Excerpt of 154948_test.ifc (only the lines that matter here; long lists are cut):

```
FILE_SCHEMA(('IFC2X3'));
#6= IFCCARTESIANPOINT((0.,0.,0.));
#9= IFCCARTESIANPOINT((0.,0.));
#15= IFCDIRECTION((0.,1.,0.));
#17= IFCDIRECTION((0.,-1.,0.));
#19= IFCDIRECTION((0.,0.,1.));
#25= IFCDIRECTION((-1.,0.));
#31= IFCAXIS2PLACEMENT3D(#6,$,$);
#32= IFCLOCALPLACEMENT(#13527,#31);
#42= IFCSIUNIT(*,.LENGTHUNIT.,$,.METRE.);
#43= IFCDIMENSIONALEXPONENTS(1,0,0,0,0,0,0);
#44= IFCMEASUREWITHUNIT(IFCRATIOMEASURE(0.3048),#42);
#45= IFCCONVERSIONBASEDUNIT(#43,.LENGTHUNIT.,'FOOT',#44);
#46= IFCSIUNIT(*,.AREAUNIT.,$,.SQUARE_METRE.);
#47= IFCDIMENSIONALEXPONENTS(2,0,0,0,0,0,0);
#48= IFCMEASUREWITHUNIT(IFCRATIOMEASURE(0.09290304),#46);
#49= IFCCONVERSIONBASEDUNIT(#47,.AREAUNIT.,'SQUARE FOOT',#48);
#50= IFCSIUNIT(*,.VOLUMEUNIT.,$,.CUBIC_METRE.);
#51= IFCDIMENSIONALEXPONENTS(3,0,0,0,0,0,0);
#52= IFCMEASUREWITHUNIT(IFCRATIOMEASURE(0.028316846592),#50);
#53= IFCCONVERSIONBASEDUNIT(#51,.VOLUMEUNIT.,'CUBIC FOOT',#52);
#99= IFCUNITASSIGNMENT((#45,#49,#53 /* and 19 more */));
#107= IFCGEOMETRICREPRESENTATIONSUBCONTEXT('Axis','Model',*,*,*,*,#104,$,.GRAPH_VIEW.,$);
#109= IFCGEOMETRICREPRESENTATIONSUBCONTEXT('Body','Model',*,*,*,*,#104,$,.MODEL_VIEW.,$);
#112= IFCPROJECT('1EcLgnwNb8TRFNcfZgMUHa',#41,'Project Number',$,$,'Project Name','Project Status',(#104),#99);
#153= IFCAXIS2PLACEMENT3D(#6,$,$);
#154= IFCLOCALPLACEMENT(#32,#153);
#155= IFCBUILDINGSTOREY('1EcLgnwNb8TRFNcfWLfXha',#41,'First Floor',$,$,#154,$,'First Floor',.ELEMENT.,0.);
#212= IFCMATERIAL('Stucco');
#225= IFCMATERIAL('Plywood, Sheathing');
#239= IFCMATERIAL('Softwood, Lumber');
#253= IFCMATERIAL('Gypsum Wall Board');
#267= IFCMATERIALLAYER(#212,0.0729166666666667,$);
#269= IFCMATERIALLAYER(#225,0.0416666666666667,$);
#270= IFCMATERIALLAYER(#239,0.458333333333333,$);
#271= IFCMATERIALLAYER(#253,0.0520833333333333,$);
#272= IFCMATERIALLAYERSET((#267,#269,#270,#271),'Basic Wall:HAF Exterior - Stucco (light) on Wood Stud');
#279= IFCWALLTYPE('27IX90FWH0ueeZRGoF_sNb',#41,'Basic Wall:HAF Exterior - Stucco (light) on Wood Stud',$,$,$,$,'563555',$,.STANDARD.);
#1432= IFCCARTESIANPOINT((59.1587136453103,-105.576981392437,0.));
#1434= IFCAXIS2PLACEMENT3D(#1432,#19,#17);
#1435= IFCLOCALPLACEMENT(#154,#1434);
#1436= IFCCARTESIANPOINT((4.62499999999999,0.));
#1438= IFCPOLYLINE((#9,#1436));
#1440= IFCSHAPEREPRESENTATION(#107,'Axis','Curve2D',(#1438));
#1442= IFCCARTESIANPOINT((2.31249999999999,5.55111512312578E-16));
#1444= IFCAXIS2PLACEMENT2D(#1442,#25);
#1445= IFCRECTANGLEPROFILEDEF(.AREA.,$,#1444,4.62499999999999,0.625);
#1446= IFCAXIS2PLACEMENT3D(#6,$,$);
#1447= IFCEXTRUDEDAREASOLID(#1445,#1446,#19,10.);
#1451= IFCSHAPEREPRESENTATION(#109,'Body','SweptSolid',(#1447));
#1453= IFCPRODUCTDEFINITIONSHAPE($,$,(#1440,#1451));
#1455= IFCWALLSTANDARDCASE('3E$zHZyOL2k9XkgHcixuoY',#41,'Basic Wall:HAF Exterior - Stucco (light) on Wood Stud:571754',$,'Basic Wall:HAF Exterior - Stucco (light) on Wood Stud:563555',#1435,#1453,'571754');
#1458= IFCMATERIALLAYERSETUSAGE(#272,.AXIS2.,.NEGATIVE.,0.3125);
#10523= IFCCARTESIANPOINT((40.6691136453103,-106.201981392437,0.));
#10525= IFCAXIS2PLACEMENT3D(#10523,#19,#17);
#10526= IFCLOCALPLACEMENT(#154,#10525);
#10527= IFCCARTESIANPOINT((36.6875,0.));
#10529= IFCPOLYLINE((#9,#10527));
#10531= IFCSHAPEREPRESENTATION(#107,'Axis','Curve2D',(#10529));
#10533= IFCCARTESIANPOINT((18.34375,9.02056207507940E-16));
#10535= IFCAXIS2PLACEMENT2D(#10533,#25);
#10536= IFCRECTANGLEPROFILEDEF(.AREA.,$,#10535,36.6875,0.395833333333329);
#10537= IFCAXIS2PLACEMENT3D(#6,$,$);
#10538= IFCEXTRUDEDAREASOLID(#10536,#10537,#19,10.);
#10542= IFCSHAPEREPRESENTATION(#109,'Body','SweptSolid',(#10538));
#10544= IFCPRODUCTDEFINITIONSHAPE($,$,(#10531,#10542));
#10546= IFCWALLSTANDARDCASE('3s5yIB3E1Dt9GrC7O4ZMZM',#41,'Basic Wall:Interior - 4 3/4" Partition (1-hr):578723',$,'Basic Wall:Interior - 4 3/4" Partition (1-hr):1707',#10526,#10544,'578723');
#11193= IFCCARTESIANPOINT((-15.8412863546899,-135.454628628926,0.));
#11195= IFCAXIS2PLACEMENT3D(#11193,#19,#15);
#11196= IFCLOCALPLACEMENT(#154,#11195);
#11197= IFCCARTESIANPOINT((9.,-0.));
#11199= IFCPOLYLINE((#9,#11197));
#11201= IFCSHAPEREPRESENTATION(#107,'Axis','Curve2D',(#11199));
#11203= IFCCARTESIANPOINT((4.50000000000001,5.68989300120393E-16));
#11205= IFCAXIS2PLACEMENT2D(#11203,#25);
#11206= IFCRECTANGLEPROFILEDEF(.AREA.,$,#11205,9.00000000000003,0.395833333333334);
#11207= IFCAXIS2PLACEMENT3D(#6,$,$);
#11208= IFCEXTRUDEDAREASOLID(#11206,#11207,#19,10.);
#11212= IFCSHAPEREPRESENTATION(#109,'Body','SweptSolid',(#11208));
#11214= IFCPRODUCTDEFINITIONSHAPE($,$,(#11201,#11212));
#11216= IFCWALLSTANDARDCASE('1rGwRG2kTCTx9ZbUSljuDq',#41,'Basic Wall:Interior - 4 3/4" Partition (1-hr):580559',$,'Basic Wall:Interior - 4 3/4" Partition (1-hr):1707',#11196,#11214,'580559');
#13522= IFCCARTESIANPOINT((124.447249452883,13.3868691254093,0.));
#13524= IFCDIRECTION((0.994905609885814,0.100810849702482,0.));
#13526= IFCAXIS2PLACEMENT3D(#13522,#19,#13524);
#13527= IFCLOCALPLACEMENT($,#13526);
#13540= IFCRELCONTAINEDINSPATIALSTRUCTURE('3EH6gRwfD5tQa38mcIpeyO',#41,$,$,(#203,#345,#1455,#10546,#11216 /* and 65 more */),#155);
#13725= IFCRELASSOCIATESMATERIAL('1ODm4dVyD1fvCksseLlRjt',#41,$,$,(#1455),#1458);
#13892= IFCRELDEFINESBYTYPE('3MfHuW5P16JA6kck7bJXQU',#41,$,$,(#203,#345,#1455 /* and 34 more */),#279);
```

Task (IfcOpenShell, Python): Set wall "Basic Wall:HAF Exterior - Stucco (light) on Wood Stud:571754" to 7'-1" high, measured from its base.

```python
import ifcopenshell
import ifcopenshell.geom
import ifcopenshell.util.representation
import ifcopenshell.util.shape
import ifcopenshell.util.unit

model = ifcopenshell.open("154948_test.ifc")
unit_scale = ifcopenshell.util.unit.calculate_unit_scale(model)
settings = ifcopenshell.geom.settings()


def volume(element):
    """Net volume in cubic metres, openings subtracted."""
    shape = ifcopenshell.geom.create_shape(settings, element)
    return ifcopenshell.util.shape.get_volume(shape.geometry)


wall = model.by_guid("3E$zHZyOL2k9XkgHcixuoY")
before = volume(wall)

body = ifcopenshell.util.representation.get_representation(wall, "Model", "Body")
solid = body.Items[0]
old_height = solid.Depth
solid.Depth = 85 * 0.0254 / unit_scale
after = volume(wall)

print(f"height {old_height:g} -> {solid.Depth:g}, volume {before:.3f} -> {after:.3f} m3")

model.write("154948_test_edited.ifc")
```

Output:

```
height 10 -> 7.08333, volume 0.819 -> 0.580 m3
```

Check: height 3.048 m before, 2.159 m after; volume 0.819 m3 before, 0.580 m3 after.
